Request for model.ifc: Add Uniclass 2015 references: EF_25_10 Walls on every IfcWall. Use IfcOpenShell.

First a look at what the model holds.

```python
import ifcopenshell

model = ifcopenshell.open("model.ifc")
print(model.schema)
print("classifications:", [c.Name for c in model.by_type("IfcClassification")])
for ifc_class in ("IfcDoor", "IfcRoof", "IfcStair", "IfcWall", "IfcWindow"):
    print(ifc_class, len(model.by_type(ifc_class)))
```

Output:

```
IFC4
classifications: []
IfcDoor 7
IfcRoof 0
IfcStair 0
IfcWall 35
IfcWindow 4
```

```python
import ifcopenshell
import ifcopenshell.api.classification

model = ifcopenshell.open("model.ifc")

system = ifcopenshell.api.classification.add_classification(model, classification="Uniclass 2015")

codes = {
    "IfcWall": ("EF_25_10", "Walls"),
}
for ifc_class, (code, name) in codes.items():
    products = model.by_type(ifc_class)
    ifcopenshell.api.classification.add_reference(
        model, products=products, classification=system, identification=code, name=name
    )
    print(code, len(products))

model.write("model_updated.ifc")
```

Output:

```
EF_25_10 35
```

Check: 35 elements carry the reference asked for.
